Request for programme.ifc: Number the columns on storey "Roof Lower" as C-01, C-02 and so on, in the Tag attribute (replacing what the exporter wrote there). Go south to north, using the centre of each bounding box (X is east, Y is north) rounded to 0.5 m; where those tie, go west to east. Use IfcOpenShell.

First a look at what the model holds.

```python
import ifcopenshell
import ifcopenshell.util.element
import ifcopenshell.util.placement

model = ifcopenshell.open("programme.ifc")
print(model.schema)
storey = next(s for s in model.by_type("IfcBuildingStorey") if s.Name == "Roof Lower")
columns = [e for e in ifcopenshell.util.element.get_decomposition(storey) if e.is_a("IfcColumn")]
for e in sorted(columns, key=lambda e: e.id()):
    origin = ifcopenshell.util.placement.get_local_placement(e.ObjectPlacement)[:3, 3]
    print(e.id(), e.Tag, e.Name, origin.round(2) + 0.0, sep=" | ")
```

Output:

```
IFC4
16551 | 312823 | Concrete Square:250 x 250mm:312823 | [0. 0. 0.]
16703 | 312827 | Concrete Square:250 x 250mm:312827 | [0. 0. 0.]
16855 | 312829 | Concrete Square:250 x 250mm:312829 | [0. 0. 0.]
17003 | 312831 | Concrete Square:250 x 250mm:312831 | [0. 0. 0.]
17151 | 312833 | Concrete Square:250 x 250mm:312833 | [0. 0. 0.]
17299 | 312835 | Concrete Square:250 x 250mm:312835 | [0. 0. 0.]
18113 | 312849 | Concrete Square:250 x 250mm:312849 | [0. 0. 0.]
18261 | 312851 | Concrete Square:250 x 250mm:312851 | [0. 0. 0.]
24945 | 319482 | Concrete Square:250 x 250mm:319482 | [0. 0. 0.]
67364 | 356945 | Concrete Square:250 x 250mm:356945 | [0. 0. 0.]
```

```python
import ifcopenshell
import ifcopenshell.geom
import ifcopenshell.util.element
import ifcopenshell.util.shape

model = ifcopenshell.open("programme.ifc")
settings = ifcopenshell.geom.settings()
settings.set("use-world-coords", True)


def centre(element):
    shape = ifcopenshell.geom.create_shape(settings, element)
    return ifcopenshell.util.shape.get_bbox_centroid(shape.geometry)


storey = next(s for s in model.by_type("IfcBuildingStorey") if s.Name == "Roof Lower")
columns = [e for e in ifcopenshell.util.element.get_decomposition(storey) if e.is_a("IfcColumn")]

# Insertion points can sit at a corner or the storey origin, so sort by the geometry (in metres).
centres = {e: centre(e) for e in columns}
columns.sort(key=lambda e: (round(centres[e][1] / 0.5), centres[e][0]))

for i, e in enumerate(columns, start=1):
    number = f"C-{i:02d}"
    e.Tag = number
    print(e.id(), number)

model.write("programme_updated.ifc")
```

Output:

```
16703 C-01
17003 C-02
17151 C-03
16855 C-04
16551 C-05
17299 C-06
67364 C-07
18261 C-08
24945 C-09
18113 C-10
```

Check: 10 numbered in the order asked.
